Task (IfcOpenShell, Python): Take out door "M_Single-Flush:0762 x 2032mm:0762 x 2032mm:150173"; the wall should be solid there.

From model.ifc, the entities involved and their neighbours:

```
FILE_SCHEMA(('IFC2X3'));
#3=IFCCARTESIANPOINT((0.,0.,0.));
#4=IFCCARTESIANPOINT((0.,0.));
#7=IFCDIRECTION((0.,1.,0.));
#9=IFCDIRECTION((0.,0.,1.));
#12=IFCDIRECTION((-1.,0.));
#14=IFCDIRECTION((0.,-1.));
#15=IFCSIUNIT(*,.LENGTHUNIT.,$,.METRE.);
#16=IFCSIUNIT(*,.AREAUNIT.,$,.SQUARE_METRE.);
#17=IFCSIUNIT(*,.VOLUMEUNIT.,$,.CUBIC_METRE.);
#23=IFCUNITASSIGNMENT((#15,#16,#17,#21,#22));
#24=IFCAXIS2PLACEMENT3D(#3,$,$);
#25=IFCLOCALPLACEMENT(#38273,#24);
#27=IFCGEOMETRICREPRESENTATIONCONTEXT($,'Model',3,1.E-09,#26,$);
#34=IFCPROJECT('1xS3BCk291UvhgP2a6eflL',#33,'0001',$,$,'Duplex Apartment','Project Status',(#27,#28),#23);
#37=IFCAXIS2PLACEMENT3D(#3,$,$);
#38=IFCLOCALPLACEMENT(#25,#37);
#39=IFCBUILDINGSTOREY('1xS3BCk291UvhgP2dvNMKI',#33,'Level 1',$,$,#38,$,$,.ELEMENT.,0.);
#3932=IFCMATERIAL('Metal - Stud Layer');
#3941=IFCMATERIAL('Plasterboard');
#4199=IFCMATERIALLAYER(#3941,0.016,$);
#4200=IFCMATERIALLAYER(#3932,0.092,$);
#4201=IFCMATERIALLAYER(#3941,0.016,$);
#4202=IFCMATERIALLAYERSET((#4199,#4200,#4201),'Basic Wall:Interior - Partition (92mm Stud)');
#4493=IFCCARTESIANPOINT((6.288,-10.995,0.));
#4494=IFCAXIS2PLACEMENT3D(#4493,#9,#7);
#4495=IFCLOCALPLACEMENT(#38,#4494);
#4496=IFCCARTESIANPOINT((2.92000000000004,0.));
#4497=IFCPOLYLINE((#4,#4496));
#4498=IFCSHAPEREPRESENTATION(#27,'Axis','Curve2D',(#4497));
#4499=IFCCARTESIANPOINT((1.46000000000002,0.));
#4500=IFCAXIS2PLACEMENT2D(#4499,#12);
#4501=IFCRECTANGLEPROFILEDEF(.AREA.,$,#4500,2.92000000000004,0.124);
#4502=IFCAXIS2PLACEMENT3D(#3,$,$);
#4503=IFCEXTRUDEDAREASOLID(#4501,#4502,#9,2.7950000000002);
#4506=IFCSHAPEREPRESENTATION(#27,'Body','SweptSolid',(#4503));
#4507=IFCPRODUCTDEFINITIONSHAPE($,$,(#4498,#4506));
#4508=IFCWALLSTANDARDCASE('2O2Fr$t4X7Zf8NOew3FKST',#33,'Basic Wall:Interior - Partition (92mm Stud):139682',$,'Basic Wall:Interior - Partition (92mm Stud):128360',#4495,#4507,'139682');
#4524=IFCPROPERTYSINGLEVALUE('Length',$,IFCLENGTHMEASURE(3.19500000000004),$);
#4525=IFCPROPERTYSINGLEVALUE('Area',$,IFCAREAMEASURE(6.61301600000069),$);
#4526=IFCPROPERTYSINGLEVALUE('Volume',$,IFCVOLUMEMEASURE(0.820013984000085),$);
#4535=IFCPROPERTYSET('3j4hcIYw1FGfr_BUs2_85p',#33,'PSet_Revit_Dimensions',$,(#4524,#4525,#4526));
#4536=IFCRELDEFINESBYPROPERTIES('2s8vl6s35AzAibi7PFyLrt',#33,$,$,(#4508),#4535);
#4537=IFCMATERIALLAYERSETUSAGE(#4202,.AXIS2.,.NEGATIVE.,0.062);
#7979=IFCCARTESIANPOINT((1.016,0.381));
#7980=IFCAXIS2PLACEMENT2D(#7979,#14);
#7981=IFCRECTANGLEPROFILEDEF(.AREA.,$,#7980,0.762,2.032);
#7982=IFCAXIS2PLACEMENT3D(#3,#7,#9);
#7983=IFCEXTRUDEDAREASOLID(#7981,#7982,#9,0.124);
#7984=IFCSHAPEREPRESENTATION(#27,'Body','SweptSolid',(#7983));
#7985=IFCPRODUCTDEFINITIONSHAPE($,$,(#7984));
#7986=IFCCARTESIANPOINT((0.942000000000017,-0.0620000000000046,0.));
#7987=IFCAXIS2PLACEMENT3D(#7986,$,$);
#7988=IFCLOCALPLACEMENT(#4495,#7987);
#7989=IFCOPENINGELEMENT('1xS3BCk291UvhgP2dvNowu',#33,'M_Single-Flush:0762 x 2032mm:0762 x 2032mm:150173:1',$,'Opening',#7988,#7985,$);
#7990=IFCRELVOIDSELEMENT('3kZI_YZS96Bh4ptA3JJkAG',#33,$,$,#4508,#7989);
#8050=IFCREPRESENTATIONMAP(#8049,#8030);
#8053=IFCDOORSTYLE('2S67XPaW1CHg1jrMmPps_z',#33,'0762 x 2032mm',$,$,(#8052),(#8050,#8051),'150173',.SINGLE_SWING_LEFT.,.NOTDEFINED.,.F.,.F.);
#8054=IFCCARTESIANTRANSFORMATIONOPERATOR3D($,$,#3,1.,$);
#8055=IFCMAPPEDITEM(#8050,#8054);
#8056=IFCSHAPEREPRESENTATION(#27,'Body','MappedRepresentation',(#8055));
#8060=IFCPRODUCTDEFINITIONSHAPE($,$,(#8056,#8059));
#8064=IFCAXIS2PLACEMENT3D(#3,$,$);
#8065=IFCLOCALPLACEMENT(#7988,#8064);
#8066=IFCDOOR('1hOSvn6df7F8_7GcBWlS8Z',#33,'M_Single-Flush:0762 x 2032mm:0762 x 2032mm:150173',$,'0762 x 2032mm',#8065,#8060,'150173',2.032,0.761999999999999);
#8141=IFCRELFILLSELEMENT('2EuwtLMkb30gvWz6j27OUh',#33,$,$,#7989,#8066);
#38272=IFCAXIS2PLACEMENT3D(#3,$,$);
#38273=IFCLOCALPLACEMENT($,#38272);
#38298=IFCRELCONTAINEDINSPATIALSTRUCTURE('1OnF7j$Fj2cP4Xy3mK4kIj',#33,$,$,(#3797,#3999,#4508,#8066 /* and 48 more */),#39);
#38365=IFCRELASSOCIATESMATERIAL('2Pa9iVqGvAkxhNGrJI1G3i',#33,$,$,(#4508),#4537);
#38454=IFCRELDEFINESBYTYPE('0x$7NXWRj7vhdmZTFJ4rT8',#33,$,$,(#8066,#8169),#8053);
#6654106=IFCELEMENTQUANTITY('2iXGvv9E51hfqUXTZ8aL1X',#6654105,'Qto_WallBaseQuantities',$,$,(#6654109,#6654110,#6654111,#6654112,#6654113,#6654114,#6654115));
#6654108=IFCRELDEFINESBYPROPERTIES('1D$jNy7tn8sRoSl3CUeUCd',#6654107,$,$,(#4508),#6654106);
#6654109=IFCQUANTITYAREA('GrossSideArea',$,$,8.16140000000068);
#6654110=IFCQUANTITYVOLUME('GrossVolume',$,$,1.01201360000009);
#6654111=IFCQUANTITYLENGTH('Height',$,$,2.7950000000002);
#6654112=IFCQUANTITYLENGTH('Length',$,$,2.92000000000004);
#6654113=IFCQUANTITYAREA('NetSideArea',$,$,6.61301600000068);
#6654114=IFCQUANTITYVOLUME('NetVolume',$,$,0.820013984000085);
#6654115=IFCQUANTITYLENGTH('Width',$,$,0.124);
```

```python
import ifcopenshell
import ifcopenshell.api.feature
import ifcopenshell.api.pset
import ifcopenshell.api.root
import ifcopenshell.geom
import ifcopenshell.util.element
import ifcopenshell.util.shape
import ifcopenshell.util.unit

model = ifcopenshell.open("model.ifc")
area_scale = ifcopenshell.util.unit.calculate_unit_scale(model, "AREAUNIT")
volume_scale = ifcopenshell.util.unit.calculate_unit_scale(model, "VOLUMEUNIT")
settings = ifcopenshell.geom.settings()


def volume(element):
    """Net volume in cubic metres, openings subtracted."""
    shape = ifcopenshell.geom.create_shape(settings, element)
    return ifcopenshell.util.shape.get_volume(shape.geometry)


door = model.by_id(8066)
opening = door.FillsVoids[0].RelatingOpeningElement
wall = opening.VoidsElements[0].RelatingBuildingElement
before = volume(wall)

ifcopenshell.api.root.remove_product(model, product=door)
ifcopenshell.api.feature.remove_feature(model, feature=opening)

after = volume(wall)
thickness = 0.124  # wall thickness in metres

# Update the wall's stored quantities.
pset = model.by_id(ifcopenshell.util.element.get_pset(wall, "PSet_Revit_Dimensions", should_inherit=False)["id"])
ifcopenshell.api.pset.edit_pset(model, pset=pset, properties={
    "Area": model.create_entity("IfcAreaMeasure", after / thickness / area_scale),
    "Volume": model.create_entity("IfcVolumeMeasure", after / volume_scale),
})
qto = model.by_id(ifcopenshell.util.element.get_pset(wall, "Qto_WallBaseQuantities", should_inherit=False)["id"])
ifcopenshell.api.pset.edit_qto(model, qto=qto, properties={
    "NetSideArea": after / thickness / area_scale,
    "NetVolume": after / volume_scale,
})

print(f"wall volume {before:.3f} -> {after:.3f} m3")

model.write("model_updated.ifc")
```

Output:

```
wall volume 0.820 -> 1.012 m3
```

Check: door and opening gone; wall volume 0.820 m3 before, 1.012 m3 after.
